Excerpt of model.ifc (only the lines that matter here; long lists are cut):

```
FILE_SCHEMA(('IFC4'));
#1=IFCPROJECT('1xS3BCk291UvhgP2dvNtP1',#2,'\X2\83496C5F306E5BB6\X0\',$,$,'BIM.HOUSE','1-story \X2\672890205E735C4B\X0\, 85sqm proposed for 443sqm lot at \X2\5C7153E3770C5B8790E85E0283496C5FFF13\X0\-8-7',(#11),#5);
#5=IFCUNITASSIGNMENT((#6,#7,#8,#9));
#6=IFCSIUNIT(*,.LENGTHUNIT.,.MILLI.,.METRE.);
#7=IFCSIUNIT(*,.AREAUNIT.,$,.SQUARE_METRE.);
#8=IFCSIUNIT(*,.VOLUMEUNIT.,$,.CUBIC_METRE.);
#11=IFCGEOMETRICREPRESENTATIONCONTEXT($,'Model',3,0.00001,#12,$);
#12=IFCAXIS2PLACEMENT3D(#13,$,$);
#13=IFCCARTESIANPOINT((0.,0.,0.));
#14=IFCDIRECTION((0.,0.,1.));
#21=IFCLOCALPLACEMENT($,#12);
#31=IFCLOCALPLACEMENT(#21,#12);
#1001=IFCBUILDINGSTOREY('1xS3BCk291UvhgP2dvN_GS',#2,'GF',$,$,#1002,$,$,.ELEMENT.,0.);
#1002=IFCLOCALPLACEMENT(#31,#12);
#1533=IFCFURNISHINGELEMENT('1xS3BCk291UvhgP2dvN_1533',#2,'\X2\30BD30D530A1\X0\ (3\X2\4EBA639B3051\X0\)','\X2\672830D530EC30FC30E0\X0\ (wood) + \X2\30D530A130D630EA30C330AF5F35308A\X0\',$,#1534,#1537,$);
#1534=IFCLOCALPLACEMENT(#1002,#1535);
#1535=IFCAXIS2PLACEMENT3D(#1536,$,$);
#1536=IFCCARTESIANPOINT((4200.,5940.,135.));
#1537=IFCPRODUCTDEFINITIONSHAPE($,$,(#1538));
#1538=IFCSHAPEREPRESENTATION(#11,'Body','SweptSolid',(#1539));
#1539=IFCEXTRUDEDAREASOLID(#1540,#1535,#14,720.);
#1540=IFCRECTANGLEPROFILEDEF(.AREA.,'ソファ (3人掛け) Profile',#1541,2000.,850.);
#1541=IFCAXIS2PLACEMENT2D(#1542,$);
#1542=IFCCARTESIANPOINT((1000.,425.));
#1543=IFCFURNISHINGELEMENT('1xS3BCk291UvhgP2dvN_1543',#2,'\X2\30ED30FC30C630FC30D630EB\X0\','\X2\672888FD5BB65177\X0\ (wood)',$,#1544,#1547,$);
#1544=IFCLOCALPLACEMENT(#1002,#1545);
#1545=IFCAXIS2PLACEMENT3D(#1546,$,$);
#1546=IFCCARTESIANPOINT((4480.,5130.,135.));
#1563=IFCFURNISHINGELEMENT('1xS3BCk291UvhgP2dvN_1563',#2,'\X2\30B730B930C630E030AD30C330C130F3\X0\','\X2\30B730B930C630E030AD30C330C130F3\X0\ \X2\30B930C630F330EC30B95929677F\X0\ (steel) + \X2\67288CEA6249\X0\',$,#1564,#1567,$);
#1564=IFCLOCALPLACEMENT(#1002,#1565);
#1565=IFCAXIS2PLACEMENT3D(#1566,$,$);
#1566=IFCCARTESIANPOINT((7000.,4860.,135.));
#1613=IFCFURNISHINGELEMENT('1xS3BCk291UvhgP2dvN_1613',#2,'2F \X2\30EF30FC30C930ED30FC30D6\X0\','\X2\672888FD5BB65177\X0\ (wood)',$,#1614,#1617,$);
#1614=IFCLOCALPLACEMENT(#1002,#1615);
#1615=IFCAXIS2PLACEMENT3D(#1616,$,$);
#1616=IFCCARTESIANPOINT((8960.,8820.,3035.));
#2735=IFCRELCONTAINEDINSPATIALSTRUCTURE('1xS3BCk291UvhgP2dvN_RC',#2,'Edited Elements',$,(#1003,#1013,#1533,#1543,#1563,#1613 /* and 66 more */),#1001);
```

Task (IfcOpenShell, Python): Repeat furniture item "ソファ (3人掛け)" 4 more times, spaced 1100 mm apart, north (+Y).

```python
import numpy as np
import ifcopenshell
import ifcopenshell.api.geometry
import ifcopenshell.api.root
import ifcopenshell.util.element
import ifcopenshell.util.placement
import ifcopenshell.util.unit

model = ifcopenshell.open("model.ifc")
unit_scale = ifcopenshell.util.unit.calculate_unit_scale(model)


def reuse_history(source, copy):
    """copy_class also copies each property set's owner history, people and application; keep the originals."""
    for rel in copy.IsDefinedBy:
        if rel.is_a("IfcRelDefinesByProperties") and (history := rel.RelatingPropertyDefinition.OwnerHistory):
            rel.RelatingPropertyDefinition.OwnerHistory = source.OwnerHistory
            ifcopenshell.util.element.remove_deep2(model, history)


source = model.by_guid("1xS3BCk291UvhgP2dvN_1533")
base = ifcopenshell.util.placement.get_local_placement(source.ObjectPlacement)
step = np.array([0.0, 1.0, 0.0]) * 1.1 / unit_scale

for i in range(1, 5):
    copy = ifcopenshell.api.root.copy_class(model, product=source)
    copy.Representation = ifcopenshell.util.element.copy_deep(
        model, source.Representation, exclude=["IfcGeometricRepresentationContext", "IfcRepresentationMap"]
    )
    reuse_history(source, copy)
    matrix = base.copy()
    matrix[:3, 3] += i * step
    print("added at", matrix[:3, 3].round(3) + 0.0)
    ifcopenshell.api.geometry.edit_object_placement(model, product=copy, matrix=matrix, is_si=False)

model.write("model-out.ifc")
```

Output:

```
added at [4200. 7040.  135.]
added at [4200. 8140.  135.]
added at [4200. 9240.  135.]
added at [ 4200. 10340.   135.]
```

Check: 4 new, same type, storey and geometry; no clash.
